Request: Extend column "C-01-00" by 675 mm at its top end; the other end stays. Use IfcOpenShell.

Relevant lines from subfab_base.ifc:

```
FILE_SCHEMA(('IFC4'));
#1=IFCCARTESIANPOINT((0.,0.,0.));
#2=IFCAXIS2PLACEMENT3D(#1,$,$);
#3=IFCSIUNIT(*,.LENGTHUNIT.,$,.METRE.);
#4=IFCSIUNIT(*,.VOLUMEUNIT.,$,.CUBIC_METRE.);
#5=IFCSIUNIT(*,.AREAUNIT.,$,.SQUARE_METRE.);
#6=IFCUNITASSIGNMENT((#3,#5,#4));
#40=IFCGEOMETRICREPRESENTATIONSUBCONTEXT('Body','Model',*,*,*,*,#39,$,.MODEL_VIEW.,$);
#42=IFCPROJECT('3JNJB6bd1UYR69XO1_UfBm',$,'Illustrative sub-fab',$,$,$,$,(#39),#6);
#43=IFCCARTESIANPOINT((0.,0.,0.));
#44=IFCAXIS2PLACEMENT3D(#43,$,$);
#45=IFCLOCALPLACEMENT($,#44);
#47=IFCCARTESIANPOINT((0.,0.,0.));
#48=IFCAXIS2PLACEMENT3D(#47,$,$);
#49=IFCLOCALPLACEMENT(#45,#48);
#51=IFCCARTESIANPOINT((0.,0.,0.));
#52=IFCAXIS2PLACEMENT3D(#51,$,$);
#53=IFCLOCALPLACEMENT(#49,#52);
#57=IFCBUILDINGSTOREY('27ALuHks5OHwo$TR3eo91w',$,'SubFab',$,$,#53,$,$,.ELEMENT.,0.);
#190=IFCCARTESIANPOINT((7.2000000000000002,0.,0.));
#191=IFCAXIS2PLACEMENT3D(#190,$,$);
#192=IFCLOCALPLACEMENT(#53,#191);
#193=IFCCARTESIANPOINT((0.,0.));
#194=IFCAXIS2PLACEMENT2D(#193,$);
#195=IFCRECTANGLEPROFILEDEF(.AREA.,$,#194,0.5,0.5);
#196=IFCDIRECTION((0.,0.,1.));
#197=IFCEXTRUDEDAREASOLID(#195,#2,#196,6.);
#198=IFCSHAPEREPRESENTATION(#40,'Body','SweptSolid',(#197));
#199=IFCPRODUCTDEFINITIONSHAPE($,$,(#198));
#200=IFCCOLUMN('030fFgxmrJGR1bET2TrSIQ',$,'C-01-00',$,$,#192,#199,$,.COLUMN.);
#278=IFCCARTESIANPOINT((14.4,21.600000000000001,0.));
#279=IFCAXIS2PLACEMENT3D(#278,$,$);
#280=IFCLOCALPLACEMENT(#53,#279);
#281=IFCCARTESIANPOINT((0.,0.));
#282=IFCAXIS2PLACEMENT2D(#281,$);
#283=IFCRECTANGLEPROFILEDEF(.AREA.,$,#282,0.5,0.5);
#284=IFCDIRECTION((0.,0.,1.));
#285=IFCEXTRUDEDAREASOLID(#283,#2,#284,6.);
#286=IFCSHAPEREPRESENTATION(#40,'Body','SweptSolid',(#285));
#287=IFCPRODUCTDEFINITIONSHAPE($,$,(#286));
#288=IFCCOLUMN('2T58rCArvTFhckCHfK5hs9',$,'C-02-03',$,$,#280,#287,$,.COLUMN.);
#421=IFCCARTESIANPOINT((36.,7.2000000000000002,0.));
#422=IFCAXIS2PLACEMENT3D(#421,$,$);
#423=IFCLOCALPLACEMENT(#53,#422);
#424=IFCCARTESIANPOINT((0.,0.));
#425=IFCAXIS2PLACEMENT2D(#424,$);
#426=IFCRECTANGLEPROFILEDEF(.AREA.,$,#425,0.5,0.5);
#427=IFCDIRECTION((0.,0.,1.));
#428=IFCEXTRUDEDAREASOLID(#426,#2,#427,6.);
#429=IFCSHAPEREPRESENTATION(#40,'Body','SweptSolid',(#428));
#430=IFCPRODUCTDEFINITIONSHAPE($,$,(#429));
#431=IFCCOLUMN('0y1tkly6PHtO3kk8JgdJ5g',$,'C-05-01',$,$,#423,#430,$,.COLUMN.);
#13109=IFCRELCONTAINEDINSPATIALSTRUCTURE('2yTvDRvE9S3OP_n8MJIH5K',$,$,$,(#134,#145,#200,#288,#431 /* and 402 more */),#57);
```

```python
import ifcopenshell
import ifcopenshell.util.representation
import ifcopenshell.util.unit

model = ifcopenshell.open("subfab_base.ifc")
unit_scale = ifcopenshell.util.unit.calculate_unit_scale(model)

member = model.by_guid("030fFgxmrJGR1bET2TrSIQ")
change = 0.675 / unit_scale

# The extrusion runs towards the end named, so only its depth changes.
body = ifcopenshell.util.representation.get_representation(member, "Model", "Body")
solid = body.Items[0]
old_length = solid.Depth
solid.Depth += change

print(f"length {old_length:g} -> {solid.Depth:g}")

model.write("subfab_base_v2.ifc")
```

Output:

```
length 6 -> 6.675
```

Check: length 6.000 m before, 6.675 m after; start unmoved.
